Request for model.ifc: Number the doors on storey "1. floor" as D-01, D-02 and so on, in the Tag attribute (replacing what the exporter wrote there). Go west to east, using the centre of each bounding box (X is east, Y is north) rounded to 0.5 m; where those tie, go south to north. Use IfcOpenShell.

First a look at what the model holds.

```python
import ifcopenshell
import ifcopenshell.util.element
import ifcopenshell.util.placement

model = ifcopenshell.open("model.ifc")
print(model.schema)
storey = next(s for s in model.by_type("IfcBuildingStorey") if s.Name == "1. floor")
doors = [e for e in ifcopenshell.util.element.get_decomposition(storey) if e.is_a("IfcDoor")]
for e in sorted(doors, key=lambda e: e.id()):
    origin = ifcopenshell.util.placement.get_local_placement(e.ObjectPlacement)[:3, 3]
    print(e.id(), e.Tag, e.Name, origin.round(2) + 0.0, sep=" | ")
```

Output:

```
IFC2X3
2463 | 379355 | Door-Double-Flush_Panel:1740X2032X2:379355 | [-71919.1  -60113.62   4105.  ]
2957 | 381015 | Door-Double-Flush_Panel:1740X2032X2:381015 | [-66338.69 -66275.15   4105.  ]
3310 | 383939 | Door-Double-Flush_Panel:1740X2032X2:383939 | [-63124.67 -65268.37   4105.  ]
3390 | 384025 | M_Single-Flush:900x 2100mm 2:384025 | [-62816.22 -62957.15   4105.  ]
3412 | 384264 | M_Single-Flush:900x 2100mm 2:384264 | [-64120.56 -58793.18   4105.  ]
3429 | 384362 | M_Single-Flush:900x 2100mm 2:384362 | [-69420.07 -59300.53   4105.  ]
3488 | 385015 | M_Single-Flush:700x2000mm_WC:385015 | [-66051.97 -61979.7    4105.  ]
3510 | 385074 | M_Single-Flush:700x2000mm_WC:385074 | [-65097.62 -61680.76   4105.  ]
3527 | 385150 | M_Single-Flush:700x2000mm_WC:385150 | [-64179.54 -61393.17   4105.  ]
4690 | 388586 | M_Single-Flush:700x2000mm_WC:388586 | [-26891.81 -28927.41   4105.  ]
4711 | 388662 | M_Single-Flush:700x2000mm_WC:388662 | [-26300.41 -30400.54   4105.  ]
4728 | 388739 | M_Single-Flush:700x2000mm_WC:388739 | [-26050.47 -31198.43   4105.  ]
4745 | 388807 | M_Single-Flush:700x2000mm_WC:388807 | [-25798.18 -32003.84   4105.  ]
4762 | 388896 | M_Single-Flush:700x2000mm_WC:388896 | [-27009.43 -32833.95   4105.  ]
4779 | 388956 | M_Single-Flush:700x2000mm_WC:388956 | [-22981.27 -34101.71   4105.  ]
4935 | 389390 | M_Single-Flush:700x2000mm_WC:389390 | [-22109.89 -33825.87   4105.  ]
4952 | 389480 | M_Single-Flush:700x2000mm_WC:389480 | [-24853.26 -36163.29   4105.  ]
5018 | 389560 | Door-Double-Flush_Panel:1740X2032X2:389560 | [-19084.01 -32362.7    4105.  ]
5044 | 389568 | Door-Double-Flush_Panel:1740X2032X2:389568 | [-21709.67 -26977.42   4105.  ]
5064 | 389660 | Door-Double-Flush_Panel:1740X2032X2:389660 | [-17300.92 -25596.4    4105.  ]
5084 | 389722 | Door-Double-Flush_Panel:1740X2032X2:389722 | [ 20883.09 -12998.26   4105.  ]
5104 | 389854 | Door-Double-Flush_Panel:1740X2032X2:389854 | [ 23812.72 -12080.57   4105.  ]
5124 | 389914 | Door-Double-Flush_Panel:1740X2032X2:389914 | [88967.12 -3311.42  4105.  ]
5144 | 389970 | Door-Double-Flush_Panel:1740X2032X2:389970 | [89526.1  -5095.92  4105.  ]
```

```python
import ifcopenshell
import ifcopenshell.geom
import ifcopenshell.util.element
import ifcopenshell.util.shape

model = ifcopenshell.open("model.ifc")
settings = ifcopenshell.geom.settings()
settings.set("use-world-coords", True)


def centre(element):
    shape = ifcopenshell.geom.create_shape(settings, element)
    return ifcopenshell.util.shape.get_bbox_centroid(shape.geometry)


storey = next(s for s in model.by_type("IfcBuildingStorey") if s.Name == "1. floor")
doors = [e for e in ifcopenshell.util.element.get_decomposition(storey) if e.is_a("IfcDoor")]

# Insertion points can sit at a corner or the storey origin, so sort by the geometry (in metres).
centres = {e: centre(e) for e in doors}
doors.sort(key=lambda e: (round(centres[e][0] / 0.5), centres[e][1]))

for i, e in enumerate(doors, start=1):
    number = f"D-{i:02d}"
    e.Tag = number
    print(e.id(), number)

model.write("model_edited.ifc")
```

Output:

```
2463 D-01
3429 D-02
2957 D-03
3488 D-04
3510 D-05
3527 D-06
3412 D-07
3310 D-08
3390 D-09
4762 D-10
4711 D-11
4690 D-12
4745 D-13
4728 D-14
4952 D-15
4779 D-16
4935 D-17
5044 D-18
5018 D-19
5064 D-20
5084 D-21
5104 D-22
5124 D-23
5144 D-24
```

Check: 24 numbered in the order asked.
